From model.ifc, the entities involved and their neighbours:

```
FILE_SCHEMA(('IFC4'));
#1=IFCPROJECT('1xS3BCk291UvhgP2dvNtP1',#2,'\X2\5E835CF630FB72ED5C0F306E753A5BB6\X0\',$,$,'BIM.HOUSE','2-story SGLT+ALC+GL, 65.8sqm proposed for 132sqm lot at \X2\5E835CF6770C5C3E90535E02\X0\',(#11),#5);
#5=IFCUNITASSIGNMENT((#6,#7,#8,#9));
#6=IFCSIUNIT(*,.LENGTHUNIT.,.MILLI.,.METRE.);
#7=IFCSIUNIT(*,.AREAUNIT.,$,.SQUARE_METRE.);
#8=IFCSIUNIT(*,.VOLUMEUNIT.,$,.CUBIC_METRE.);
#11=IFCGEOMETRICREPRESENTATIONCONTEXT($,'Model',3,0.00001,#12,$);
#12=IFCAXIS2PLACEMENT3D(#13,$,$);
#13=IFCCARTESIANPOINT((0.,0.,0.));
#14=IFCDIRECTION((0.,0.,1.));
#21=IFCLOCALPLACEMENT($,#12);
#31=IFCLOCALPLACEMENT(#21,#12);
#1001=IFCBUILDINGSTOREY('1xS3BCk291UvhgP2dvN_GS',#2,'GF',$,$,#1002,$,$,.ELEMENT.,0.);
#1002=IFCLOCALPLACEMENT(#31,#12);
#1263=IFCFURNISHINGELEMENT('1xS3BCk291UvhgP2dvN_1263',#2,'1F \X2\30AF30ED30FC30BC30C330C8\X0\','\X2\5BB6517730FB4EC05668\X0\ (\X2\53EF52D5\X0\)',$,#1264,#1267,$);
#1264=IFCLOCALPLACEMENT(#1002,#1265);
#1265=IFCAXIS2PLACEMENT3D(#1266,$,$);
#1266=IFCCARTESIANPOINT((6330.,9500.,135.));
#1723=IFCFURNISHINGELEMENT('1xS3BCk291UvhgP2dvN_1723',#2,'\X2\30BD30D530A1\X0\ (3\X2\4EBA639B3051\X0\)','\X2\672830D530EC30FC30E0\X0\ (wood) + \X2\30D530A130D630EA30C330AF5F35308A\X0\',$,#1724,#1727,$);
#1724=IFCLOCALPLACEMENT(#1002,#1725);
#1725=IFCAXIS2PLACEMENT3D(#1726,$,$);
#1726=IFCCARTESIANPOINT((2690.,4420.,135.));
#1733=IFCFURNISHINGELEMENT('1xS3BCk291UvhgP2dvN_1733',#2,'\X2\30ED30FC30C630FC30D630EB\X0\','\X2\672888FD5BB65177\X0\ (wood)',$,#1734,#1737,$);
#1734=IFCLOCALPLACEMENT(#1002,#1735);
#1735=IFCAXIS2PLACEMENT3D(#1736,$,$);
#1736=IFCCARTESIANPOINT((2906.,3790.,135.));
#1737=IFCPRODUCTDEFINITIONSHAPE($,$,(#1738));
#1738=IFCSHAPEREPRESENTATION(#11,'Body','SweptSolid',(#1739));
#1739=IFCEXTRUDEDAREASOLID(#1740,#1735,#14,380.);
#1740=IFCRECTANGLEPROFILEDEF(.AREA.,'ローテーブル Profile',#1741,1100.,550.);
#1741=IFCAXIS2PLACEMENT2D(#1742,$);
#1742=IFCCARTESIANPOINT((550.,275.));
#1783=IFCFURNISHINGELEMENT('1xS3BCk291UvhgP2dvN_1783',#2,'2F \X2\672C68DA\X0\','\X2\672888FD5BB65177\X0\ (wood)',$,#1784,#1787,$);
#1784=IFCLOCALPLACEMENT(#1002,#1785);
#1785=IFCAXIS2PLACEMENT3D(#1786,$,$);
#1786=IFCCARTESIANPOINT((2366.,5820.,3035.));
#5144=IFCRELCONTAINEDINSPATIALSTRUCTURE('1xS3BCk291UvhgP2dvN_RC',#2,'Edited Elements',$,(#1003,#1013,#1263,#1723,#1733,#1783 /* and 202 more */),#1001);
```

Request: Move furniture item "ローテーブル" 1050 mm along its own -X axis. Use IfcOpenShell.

```python
import ifcopenshell
import ifcopenshell.api.geometry
import ifcopenshell.util.placement

model = ifcopenshell.open("model.ifc")

item = model.by_id(1733)
matrix = ifcopenshell.util.placement.get_local_placement(item.ObjectPlacement)
matrix[:3, 3] -= matrix[:3, 0] * 1050.0
ifcopenshell.api.geometry.edit_object_placement(model, product=item, matrix=matrix, is_si=False)

print(ifcopenshell.util.placement.get_local_placement(item.ObjectPlacement).round(3) + 0.0)

model.write("model_v2.ifc")
```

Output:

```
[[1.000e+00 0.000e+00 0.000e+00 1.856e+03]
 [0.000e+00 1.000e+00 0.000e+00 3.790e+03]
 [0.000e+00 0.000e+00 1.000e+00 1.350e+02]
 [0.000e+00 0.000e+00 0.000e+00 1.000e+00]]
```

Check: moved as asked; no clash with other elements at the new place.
